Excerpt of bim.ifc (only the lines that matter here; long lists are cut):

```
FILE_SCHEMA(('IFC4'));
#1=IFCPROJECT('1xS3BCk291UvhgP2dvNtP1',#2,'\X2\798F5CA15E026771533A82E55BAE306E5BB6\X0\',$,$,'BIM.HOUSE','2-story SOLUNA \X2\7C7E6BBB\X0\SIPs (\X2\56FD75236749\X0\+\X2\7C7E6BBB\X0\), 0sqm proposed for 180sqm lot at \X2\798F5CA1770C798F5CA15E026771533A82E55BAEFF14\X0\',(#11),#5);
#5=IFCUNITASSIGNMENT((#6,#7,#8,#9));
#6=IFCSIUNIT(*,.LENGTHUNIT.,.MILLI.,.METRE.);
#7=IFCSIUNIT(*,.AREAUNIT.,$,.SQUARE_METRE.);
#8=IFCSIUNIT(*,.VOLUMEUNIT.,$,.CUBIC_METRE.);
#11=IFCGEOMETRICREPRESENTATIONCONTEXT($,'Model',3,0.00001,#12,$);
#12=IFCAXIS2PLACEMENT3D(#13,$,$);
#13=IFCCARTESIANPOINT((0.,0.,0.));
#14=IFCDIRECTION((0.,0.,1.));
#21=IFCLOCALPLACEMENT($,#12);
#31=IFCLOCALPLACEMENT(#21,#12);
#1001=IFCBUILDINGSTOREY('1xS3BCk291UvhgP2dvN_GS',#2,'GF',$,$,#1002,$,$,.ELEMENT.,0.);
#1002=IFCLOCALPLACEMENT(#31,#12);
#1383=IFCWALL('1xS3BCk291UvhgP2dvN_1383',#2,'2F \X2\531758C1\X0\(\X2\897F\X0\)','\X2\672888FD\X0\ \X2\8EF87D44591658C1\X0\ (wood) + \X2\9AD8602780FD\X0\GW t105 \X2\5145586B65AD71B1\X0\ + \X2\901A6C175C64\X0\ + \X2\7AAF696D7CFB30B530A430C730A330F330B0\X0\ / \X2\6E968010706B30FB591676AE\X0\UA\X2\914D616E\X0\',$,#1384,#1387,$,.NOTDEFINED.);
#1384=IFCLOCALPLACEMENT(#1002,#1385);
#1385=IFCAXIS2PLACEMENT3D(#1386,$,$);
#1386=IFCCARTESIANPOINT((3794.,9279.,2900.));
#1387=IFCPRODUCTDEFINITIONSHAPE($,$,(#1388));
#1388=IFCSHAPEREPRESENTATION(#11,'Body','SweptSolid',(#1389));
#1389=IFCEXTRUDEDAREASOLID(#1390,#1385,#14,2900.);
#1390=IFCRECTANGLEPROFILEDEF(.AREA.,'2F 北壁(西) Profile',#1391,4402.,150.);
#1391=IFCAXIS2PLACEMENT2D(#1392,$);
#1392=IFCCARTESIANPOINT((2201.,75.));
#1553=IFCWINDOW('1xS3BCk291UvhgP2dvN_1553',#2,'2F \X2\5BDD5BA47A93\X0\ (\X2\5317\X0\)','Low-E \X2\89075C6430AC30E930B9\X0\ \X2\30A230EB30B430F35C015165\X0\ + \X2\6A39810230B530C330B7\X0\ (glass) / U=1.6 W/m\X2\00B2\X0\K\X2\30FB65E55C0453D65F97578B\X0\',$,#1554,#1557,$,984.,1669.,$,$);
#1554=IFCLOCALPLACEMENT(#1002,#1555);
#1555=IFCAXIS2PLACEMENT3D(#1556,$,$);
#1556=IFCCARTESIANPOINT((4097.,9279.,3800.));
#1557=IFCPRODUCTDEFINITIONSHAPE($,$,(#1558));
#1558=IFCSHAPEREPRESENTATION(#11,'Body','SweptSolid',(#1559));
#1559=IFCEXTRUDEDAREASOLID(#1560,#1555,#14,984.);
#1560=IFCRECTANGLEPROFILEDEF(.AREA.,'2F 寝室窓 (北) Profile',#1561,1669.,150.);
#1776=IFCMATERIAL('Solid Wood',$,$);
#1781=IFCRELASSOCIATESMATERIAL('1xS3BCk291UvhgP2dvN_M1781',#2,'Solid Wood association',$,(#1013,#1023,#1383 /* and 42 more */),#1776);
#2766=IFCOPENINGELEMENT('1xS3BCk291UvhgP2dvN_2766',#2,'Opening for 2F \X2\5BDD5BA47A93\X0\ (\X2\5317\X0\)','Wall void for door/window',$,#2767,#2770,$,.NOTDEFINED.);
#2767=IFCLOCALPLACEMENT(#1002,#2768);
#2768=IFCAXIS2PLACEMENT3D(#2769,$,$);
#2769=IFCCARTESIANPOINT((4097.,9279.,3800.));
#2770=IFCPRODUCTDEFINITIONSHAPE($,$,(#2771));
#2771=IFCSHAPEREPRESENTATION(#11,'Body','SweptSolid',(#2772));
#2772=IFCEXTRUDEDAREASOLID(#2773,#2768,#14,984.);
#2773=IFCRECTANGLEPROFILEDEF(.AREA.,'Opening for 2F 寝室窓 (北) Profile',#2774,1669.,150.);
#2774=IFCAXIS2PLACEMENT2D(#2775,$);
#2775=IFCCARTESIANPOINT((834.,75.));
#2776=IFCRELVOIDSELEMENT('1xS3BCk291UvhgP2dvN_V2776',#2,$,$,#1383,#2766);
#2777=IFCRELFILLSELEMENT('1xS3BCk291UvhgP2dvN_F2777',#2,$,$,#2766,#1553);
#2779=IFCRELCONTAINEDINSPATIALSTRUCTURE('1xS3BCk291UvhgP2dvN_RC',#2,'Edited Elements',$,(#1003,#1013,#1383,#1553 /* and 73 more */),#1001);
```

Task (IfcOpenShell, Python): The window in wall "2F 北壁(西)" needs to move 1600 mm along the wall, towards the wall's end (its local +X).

```python
import ifcopenshell
import ifcopenshell.api.geometry
import ifcopenshell.util.placement
import ifcopenshell.util.unit

model = ifcopenshell.open("bim.ifc")
unit_scale = ifcopenshell.util.unit.calculate_unit_scale(model)

window = model.by_guid("1xS3BCk291UvhgP2dvN_1553")
opening = window.FillsVoids[0].RelatingOpeningElement
wall = opening.VoidsElements[0].RelatingBuildingElement

wall_matrix = ifcopenshell.util.placement.get_local_placement(wall.ObjectPlacement)
shift = wall_matrix[:3, 0] * 1.6 / unit_scale
before = ifcopenshell.util.placement.get_local_placement(window.ObjectPlacement)[:3, 3].copy()

# The window is not placed relative to its opening, so move both.
for product in (opening, window):
    matrix = ifcopenshell.util.placement.get_local_placement(product.ObjectPlacement)
    matrix[:3, 3] += shift
    ifcopenshell.api.geometry.edit_object_placement(model, product=product, matrix=matrix, is_si=False)

after = ifcopenshell.util.placement.get_local_placement(window.ObjectPlacement)[:3, 3]
print("window moved by", (after - before).round(3) + 0.0)

model.write("bim-out.ifc")
```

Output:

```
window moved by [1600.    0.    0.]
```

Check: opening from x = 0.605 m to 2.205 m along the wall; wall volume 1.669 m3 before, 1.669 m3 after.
